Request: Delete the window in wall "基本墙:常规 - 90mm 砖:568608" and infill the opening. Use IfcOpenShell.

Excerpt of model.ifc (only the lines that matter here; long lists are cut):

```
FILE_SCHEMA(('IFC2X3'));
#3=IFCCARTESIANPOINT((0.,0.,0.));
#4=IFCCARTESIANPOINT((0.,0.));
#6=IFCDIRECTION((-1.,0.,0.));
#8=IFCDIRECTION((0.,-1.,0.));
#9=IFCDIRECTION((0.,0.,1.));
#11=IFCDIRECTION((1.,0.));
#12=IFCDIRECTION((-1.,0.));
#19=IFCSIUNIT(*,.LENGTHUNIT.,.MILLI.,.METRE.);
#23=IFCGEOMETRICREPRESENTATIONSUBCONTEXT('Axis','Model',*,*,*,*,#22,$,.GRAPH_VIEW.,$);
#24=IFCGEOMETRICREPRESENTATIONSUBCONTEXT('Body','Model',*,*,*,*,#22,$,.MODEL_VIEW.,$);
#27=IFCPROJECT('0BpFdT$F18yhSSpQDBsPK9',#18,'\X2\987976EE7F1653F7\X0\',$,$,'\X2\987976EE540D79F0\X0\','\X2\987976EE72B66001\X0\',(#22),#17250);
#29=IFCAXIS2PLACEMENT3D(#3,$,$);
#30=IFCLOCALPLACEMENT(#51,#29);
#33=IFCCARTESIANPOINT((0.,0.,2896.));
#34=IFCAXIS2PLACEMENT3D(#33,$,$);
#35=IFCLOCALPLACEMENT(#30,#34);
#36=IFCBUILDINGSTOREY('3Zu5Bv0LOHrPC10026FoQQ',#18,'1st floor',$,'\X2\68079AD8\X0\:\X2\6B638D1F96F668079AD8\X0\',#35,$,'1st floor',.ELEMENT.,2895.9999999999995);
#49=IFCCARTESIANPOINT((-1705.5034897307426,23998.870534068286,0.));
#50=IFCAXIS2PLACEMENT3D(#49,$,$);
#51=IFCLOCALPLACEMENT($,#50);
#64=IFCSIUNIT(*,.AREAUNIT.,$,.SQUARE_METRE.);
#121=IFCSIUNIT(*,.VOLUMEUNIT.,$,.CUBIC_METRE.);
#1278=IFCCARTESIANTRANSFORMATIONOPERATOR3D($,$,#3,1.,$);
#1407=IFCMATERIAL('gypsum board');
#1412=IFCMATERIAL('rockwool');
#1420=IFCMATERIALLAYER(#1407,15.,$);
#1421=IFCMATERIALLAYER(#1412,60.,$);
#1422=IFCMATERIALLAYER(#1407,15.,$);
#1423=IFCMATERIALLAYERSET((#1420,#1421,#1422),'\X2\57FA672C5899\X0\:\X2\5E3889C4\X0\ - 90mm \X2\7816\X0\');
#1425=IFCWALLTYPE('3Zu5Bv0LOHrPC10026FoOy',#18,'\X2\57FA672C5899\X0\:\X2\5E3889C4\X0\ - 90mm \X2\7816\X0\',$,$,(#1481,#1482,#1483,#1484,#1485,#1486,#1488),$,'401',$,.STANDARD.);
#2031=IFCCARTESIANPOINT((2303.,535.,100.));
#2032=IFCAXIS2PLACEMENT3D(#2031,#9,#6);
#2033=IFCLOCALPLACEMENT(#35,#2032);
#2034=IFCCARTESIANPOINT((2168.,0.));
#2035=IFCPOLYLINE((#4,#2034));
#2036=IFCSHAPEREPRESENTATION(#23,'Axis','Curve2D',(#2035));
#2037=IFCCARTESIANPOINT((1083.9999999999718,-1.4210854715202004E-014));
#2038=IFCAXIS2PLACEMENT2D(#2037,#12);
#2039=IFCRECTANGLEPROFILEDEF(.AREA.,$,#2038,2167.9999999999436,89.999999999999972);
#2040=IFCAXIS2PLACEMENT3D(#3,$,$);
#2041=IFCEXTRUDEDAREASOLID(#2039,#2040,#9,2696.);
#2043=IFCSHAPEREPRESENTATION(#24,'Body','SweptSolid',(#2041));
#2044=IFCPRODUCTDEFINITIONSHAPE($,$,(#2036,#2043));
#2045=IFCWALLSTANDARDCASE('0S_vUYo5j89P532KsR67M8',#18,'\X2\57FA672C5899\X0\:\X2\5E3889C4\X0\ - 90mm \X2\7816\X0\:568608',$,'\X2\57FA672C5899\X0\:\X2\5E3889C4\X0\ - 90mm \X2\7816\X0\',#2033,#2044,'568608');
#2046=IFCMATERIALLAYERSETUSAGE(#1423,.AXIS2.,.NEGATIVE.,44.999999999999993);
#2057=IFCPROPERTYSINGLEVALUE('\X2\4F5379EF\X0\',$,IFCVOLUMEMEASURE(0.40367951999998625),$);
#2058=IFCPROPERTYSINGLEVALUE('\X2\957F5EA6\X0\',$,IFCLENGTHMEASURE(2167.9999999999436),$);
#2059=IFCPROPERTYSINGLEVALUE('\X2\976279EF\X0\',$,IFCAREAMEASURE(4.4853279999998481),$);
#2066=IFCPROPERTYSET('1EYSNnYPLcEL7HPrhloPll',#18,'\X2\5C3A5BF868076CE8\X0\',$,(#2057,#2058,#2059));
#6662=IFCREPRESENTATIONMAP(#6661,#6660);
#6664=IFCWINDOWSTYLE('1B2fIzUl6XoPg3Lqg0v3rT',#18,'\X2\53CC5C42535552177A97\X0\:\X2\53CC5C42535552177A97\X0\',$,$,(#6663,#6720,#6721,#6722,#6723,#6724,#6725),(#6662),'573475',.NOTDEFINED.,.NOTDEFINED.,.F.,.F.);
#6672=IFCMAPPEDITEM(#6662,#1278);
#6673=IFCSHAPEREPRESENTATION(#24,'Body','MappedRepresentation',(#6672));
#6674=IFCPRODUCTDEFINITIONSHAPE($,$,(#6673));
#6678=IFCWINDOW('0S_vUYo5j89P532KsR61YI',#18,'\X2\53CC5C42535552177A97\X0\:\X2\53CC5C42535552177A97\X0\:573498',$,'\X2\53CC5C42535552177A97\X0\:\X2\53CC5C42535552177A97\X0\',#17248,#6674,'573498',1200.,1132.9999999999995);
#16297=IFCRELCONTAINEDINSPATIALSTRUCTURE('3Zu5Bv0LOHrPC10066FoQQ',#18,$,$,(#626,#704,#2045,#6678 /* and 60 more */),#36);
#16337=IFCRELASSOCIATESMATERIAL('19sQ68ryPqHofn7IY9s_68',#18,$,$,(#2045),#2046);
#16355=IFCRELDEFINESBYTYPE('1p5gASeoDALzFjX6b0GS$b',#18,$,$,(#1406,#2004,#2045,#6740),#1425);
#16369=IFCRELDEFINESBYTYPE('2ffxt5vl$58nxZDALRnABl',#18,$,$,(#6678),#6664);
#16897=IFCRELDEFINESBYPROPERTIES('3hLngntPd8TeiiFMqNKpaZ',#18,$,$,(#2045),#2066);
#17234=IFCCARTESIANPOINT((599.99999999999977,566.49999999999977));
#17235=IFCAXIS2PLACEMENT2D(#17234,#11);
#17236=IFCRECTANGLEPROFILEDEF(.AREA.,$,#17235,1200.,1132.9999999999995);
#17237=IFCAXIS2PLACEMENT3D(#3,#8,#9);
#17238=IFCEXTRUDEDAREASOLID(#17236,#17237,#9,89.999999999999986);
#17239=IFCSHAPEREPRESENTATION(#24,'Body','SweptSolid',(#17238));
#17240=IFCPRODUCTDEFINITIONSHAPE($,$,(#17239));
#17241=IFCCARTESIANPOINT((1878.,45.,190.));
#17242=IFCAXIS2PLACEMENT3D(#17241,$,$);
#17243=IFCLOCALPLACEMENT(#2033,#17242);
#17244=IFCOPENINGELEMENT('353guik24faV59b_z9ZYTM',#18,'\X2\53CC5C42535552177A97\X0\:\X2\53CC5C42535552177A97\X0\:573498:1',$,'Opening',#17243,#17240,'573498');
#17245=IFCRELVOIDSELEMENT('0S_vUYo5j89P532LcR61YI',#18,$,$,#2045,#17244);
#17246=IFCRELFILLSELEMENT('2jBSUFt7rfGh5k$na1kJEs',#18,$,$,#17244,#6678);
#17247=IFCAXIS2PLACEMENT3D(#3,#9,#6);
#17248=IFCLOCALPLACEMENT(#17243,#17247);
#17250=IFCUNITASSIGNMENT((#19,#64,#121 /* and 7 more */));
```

```python
import ifcopenshell
import ifcopenshell.api.feature
import ifcopenshell.api.pset
import ifcopenshell.api.root
import ifcopenshell.geom
import ifcopenshell.util.element
import ifcopenshell.util.shape
import ifcopenshell.util.unit

model = ifcopenshell.open("model.ifc")
area_scale = ifcopenshell.util.unit.calculate_unit_scale(model, "AREAUNIT")
volume_scale = ifcopenshell.util.unit.calculate_unit_scale(model, "VOLUMEUNIT")
settings = ifcopenshell.geom.settings()


def volume(element):
    """Net volume in cubic metres, openings subtracted."""
    shape = ifcopenshell.geom.create_shape(settings, element)
    return ifcopenshell.util.shape.get_volume(shape.geometry)


window = model.by_guid("0S_vUYo5j89P532KsR61YI")
opening = window.FillsVoids[0].RelatingOpeningElement
wall = opening.VoidsElements[0].RelatingBuildingElement
before = volume(wall)

ifcopenshell.api.root.remove_product(model, product=window)
ifcopenshell.api.feature.remove_feature(model, feature=opening)

after = volume(wall)
thickness = 0.09  # wall thickness in metres

# Update the wall's stored quantities.
pset = model.by_id(ifcopenshell.util.element.get_pset(wall, "尺寸标注", should_inherit=False)["id"])
ifcopenshell.api.pset.edit_pset(model, pset=pset, properties={
    "体积": model.create_entity("IfcVolumeMeasure", after / volume_scale),
    "面积": model.create_entity("IfcAreaMeasure", after / thickness / area_scale),
})

print(f"wall volume {before:.3f} -> {after:.3f} m3")

model.write("model_rev.ifc")
```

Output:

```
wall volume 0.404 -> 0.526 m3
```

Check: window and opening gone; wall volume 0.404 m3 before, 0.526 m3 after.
